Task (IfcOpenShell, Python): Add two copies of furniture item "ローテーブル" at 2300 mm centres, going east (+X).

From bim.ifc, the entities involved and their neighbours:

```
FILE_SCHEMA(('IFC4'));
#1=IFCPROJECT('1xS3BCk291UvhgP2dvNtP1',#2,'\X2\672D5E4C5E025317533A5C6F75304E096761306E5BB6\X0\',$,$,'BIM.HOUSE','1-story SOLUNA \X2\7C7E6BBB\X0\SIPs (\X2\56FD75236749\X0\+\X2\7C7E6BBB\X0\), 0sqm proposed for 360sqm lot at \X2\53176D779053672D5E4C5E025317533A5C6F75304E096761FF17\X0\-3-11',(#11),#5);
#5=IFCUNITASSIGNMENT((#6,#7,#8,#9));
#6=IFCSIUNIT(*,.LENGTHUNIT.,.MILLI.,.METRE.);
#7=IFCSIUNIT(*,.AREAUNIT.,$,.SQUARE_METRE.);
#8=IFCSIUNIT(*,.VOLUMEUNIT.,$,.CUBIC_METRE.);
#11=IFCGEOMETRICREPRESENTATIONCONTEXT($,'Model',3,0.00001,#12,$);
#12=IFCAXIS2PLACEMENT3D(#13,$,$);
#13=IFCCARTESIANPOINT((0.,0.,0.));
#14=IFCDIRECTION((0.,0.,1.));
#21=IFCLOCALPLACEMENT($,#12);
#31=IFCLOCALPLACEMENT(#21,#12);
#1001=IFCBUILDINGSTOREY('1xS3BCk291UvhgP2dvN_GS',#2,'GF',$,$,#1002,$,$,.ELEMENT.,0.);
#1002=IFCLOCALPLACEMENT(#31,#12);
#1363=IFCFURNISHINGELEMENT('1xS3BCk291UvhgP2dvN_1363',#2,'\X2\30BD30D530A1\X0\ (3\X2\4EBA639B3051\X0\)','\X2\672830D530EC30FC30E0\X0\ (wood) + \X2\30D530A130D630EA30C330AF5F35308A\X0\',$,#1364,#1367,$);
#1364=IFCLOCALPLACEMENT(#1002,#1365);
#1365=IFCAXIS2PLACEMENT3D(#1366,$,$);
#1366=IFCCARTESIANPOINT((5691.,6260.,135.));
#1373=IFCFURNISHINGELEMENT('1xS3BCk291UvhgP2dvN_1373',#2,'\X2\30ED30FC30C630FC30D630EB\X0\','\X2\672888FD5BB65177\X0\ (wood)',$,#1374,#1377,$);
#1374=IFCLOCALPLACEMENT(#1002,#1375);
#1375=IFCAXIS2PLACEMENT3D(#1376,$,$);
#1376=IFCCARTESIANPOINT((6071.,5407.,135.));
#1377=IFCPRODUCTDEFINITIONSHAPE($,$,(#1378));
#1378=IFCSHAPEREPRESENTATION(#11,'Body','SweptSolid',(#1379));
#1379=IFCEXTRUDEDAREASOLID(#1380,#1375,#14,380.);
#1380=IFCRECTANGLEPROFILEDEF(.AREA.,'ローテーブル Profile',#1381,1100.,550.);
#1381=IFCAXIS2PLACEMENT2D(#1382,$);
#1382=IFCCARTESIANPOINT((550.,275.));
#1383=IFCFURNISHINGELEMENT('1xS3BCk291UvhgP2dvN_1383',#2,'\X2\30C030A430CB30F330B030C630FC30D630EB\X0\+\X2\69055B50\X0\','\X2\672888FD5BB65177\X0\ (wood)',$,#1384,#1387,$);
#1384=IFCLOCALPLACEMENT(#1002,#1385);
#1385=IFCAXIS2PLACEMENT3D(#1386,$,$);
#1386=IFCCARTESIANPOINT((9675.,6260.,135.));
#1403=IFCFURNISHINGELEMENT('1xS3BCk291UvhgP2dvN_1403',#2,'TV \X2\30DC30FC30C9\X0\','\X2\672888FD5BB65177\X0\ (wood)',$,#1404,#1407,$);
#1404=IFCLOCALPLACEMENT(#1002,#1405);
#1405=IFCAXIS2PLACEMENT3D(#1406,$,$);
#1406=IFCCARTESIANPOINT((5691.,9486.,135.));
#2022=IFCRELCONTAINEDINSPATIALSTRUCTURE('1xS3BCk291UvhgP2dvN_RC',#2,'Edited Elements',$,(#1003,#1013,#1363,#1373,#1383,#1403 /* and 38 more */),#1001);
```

```python
import numpy as np
import ifcopenshell
import ifcopenshell.api.geometry
import ifcopenshell.api.root
import ifcopenshell.util.element
import ifcopenshell.util.placement
import ifcopenshell.util.unit

model = ifcopenshell.open("bim.ifc")
unit_scale = ifcopenshell.util.unit.calculate_unit_scale(model)


def reuse_history(source, copy):
    """copy_class also copies each property set's owner history, people and application; keep the originals."""
    for rel in copy.IsDefinedBy:
        if rel.is_a("IfcRelDefinesByProperties") and (history := rel.RelatingPropertyDefinition.OwnerHistory):
            rel.RelatingPropertyDefinition.OwnerHistory = source.OwnerHistory
            ifcopenshell.util.element.remove_deep2(model, history)


source = model.by_guid("1xS3BCk291UvhgP2dvN_1373")
base = ifcopenshell.util.placement.get_local_placement(source.ObjectPlacement)
step = np.array([1.0, 0.0, 0.0]) * 2.3 / unit_scale

for i in range(1, 3):
    copy = ifcopenshell.api.root.copy_class(model, product=source)
    copy.Representation = ifcopenshell.util.element.copy_deep(
        model, source.Representation, exclude=["IfcGeometricRepresentationContext", "IfcRepresentationMap"]
    )
    reuse_history(source, copy)
    matrix = base.copy()
    matrix[:3, 3] += i * step
    print("added at", matrix[:3, 3].round(3) + 0.0)
    ifcopenshell.api.geometry.edit_object_placement(model, product=copy, matrix=matrix, is_si=False)

model.write("bim-out.ifc")
```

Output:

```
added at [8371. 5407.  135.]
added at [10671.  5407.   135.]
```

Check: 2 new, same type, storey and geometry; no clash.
